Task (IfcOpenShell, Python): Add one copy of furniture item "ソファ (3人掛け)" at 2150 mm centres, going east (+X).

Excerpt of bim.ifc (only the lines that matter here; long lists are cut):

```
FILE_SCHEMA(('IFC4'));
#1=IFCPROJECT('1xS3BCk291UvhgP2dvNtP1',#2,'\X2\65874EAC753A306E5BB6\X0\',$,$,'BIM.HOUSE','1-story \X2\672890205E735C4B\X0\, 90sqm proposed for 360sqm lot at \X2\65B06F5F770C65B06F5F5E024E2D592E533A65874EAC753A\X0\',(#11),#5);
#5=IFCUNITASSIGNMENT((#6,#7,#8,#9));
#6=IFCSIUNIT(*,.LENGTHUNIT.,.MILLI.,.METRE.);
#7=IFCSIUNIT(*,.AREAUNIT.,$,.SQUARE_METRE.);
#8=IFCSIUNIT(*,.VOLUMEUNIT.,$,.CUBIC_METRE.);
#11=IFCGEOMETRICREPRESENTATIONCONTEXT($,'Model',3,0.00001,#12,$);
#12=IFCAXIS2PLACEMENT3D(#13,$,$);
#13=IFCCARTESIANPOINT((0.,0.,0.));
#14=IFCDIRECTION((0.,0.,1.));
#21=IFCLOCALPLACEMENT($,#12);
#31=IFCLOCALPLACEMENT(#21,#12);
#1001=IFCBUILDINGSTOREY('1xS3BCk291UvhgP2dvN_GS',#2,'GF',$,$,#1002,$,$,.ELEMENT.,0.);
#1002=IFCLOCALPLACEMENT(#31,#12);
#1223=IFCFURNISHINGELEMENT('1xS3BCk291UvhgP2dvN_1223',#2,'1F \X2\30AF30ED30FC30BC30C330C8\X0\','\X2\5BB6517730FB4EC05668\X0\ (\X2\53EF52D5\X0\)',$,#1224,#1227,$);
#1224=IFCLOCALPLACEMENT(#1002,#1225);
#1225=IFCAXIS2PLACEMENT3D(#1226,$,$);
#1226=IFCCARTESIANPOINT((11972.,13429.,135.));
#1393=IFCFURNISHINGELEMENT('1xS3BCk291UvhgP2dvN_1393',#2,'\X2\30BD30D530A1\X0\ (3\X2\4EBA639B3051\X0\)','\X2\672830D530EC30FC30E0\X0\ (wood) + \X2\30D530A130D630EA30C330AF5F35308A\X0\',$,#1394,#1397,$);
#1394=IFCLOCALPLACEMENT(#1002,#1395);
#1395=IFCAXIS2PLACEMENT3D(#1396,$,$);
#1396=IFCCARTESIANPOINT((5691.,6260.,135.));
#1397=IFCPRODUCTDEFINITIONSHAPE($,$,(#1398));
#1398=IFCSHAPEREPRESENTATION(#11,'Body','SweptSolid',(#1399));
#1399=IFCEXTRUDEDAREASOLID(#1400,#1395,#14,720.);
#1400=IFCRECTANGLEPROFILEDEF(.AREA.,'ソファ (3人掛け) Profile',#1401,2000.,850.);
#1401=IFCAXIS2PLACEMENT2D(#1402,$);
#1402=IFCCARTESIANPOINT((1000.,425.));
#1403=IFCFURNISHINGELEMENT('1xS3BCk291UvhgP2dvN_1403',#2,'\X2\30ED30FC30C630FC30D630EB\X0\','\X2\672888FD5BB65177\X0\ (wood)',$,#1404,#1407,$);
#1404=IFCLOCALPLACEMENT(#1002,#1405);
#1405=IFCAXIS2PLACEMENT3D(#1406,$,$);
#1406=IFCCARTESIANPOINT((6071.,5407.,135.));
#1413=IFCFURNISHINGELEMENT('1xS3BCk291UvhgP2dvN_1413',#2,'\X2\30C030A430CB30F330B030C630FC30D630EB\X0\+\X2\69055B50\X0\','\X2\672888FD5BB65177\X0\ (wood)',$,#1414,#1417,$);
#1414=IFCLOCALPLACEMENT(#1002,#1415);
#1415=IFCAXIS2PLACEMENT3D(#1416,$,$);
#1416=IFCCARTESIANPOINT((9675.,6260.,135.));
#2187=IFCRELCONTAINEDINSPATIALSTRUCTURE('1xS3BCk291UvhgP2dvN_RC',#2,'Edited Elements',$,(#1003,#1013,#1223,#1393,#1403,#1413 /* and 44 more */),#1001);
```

```python
import numpy as np
import ifcopenshell
import ifcopenshell.api.geometry
import ifcopenshell.api.root
import ifcopenshell.util.element
import ifcopenshell.util.placement
import ifcopenshell.util.unit

model = ifcopenshell.open("bim.ifc")
unit_scale = ifcopenshell.util.unit.calculate_unit_scale(model)


def reuse_history(source, copy):
    """copy_class also copies each property set's owner history, people and application; keep the originals."""
    for rel in copy.IsDefinedBy:
        if rel.is_a("IfcRelDefinesByProperties") and (history := rel.RelatingPropertyDefinition.OwnerHistory):
            rel.RelatingPropertyDefinition.OwnerHistory = source.OwnerHistory
            ifcopenshell.util.element.remove_deep2(model, history)


source = model.by_guid("1xS3BCk291UvhgP2dvN_1393")
base = ifcopenshell.util.placement.get_local_placement(source.ObjectPlacement)
step = np.array([1.0, 0.0, 0.0]) * 2.15 / unit_scale

for i in range(1, 2):
    copy = ifcopenshell.api.root.copy_class(model, product=source)
    copy.Representation = ifcopenshell.util.element.copy_deep(
        model, source.Representation, exclude=["IfcGeometricRepresentationContext", "IfcRepresentationMap"]
    )
    reuse_history(source, copy)
    matrix = base.copy()
    matrix[:3, 3] += i * step
    print("added at", matrix[:3, 3].round(3) + 0.0)
    ifcopenshell.api.geometry.edit_object_placement(model, product=copy, matrix=matrix, is_si=False)

model.write("bim_updated.ifc")
```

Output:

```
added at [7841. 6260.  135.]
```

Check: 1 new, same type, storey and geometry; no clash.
